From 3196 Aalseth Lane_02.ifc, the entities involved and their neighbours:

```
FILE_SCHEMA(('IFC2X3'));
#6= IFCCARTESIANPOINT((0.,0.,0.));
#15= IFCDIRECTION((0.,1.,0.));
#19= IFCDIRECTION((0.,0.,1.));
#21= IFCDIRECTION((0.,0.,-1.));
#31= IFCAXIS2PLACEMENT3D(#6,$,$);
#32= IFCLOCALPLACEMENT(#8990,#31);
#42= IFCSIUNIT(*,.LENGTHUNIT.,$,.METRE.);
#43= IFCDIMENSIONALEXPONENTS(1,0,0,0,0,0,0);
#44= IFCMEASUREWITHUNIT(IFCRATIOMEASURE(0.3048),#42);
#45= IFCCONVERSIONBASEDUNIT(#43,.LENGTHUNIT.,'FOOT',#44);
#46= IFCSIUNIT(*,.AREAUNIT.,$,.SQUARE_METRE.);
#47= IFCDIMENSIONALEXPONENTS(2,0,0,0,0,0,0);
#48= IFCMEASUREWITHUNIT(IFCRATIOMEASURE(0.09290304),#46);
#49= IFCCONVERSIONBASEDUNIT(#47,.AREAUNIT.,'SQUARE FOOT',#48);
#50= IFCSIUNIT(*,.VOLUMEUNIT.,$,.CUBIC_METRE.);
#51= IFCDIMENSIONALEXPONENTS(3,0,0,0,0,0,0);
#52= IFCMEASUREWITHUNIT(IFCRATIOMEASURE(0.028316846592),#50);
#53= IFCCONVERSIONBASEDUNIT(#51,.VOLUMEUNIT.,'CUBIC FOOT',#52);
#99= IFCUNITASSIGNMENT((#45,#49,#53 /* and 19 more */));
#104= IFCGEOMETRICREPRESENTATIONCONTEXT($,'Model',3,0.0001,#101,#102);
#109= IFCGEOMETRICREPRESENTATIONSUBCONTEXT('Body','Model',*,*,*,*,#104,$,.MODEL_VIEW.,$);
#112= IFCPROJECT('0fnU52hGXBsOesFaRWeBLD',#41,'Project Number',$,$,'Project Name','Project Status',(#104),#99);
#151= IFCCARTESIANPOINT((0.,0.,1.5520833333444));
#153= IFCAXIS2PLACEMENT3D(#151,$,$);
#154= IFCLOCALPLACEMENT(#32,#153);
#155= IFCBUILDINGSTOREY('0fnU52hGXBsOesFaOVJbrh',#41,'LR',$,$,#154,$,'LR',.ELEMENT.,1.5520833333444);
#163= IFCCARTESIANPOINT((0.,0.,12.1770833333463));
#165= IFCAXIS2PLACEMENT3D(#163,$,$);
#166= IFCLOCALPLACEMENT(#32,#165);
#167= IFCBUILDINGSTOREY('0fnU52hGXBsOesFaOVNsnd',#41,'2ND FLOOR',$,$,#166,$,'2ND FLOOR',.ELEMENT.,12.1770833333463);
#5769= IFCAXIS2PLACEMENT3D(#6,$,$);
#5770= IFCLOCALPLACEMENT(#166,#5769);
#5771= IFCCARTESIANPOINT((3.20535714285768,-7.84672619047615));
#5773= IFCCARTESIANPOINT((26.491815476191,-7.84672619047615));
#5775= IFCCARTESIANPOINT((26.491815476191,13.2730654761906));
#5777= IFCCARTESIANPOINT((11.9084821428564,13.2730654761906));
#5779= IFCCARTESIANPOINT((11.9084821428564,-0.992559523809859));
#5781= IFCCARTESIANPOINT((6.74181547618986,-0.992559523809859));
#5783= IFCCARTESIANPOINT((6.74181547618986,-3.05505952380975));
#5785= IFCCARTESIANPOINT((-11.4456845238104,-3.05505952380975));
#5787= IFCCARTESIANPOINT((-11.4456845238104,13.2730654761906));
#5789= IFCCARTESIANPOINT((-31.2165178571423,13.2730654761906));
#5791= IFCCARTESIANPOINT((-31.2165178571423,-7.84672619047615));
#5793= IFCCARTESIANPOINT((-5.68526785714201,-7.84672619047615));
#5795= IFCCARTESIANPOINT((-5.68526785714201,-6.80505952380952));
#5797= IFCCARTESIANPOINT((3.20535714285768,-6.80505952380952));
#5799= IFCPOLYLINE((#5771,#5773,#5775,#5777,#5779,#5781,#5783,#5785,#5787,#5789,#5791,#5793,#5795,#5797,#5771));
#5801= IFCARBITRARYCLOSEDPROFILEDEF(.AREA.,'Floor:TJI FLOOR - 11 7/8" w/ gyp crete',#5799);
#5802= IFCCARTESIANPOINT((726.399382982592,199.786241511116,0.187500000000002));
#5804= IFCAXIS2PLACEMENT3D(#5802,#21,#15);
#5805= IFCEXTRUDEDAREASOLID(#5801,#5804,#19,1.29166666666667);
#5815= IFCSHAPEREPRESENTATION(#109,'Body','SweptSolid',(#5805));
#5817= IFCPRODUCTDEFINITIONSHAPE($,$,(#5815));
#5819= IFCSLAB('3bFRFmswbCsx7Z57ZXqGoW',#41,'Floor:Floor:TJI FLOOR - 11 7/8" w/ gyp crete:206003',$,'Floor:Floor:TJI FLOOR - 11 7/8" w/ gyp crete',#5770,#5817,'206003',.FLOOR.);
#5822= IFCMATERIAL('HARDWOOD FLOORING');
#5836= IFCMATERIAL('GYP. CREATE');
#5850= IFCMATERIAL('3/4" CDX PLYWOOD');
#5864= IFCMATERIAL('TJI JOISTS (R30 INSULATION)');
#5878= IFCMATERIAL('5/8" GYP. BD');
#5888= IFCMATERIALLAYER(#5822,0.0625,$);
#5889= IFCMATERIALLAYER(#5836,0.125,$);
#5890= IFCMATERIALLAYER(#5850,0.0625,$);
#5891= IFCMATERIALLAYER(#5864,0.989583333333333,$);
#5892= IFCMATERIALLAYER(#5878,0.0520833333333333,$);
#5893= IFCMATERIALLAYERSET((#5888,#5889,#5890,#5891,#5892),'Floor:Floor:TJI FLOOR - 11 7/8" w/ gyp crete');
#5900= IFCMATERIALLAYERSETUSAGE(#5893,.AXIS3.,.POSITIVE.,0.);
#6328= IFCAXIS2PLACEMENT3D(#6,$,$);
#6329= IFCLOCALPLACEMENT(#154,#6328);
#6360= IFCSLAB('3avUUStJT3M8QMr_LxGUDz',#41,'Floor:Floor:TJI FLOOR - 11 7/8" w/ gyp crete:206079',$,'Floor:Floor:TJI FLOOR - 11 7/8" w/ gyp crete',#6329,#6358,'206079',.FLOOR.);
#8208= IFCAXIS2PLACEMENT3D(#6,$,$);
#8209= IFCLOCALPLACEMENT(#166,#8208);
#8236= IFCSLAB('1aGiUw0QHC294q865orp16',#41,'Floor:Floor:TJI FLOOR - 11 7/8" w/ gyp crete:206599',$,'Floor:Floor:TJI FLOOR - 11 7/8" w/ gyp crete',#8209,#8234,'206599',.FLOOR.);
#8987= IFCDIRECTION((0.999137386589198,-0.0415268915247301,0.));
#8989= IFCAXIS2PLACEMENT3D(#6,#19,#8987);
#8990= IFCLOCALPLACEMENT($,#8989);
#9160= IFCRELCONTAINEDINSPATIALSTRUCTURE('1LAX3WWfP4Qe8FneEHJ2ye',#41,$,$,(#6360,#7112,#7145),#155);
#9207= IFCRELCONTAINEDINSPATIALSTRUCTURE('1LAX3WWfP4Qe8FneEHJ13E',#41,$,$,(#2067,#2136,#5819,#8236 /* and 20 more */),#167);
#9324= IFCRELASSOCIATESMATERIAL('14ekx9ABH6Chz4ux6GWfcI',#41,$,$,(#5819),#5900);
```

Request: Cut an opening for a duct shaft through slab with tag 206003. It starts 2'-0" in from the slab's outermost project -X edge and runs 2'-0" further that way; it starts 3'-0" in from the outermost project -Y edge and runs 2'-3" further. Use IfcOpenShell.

```python
import numpy as np
import ifcopenshell
import ifcopenshell.api.feature
import ifcopenshell.api.geometry
import ifcopenshell.api.root
import ifcopenshell.geom
import ifcopenshell.util.placement
import ifcopenshell.util.representation
import ifcopenshell.util.shape
import ifcopenshell.util.unit

model = ifcopenshell.open("3196 Aalseth Lane_02.ifc")
unit_scale = ifcopenshell.util.unit.calculate_unit_scale(model)
settings = ifcopenshell.geom.settings()


def volume(element):
    """Net volume in cubic metres, openings subtracted."""
    shape = ifcopenshell.geom.create_shape(settings, element)
    return ifcopenshell.util.shape.get_volume(shape.geometry)


slab = model.by_guid("3bFRFmswbCsx7Z57ZXqGoW")
before = volume(slab)

# Extent in the slab's own axes, in metres. The edges named are its -X and -Y sides.
slab_shape = ifcopenshell.geom.create_shape(settings, slab)
vertices = ifcopenshell.util.shape.get_vertices(slab_shape.geometry)
x_min, y_min, bottom = vertices.min(axis=0)
top = vertices[:, 2].max()

opening = ifcopenshell.api.root.create_entity(model, ifc_class="IfcOpeningElement", name="Duct shaft opening")
context = ifcopenshell.util.representation.get_context(model, "Model", "Body", "MODEL_VIEW")
width, depth = 0.6096, 0.6858
outline = [(0.0, 0.0), (width, 0.0), (width, depth), (0.0, depth), (0.0, 0.0)]
# Overshoot both faces by 50 mm so the cut is clean.
shape = ifcopenshell.api.geometry.add_slab_representation(
    model, context=context, depth=top - bottom + 0.1, polyline=outline
)
ifcopenshell.api.geometry.assign_representation(model, product=opening, representation=shape)

matrix = ifcopenshell.util.placement.get_local_placement(slab.ObjectPlacement)
matrix[:, 3] = matrix @ np.append(np.array([x_min + 0.6096, y_min + 0.9144, bottom - 0.05]) / unit_scale, 1.0)
ifcopenshell.api.geometry.edit_object_placement(model, product=opening, matrix=matrix, is_si=False)
ifcopenshell.api.feature.add_feature(model, feature=opening, element=slab)

after = volume(slab)

print(f"slab volume {before:.3f} -> {after:.3f} m3")

model.write("3196 Aalseth Lane_02_updated.ifc")
```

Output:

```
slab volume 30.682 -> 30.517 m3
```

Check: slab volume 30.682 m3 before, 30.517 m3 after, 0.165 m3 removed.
